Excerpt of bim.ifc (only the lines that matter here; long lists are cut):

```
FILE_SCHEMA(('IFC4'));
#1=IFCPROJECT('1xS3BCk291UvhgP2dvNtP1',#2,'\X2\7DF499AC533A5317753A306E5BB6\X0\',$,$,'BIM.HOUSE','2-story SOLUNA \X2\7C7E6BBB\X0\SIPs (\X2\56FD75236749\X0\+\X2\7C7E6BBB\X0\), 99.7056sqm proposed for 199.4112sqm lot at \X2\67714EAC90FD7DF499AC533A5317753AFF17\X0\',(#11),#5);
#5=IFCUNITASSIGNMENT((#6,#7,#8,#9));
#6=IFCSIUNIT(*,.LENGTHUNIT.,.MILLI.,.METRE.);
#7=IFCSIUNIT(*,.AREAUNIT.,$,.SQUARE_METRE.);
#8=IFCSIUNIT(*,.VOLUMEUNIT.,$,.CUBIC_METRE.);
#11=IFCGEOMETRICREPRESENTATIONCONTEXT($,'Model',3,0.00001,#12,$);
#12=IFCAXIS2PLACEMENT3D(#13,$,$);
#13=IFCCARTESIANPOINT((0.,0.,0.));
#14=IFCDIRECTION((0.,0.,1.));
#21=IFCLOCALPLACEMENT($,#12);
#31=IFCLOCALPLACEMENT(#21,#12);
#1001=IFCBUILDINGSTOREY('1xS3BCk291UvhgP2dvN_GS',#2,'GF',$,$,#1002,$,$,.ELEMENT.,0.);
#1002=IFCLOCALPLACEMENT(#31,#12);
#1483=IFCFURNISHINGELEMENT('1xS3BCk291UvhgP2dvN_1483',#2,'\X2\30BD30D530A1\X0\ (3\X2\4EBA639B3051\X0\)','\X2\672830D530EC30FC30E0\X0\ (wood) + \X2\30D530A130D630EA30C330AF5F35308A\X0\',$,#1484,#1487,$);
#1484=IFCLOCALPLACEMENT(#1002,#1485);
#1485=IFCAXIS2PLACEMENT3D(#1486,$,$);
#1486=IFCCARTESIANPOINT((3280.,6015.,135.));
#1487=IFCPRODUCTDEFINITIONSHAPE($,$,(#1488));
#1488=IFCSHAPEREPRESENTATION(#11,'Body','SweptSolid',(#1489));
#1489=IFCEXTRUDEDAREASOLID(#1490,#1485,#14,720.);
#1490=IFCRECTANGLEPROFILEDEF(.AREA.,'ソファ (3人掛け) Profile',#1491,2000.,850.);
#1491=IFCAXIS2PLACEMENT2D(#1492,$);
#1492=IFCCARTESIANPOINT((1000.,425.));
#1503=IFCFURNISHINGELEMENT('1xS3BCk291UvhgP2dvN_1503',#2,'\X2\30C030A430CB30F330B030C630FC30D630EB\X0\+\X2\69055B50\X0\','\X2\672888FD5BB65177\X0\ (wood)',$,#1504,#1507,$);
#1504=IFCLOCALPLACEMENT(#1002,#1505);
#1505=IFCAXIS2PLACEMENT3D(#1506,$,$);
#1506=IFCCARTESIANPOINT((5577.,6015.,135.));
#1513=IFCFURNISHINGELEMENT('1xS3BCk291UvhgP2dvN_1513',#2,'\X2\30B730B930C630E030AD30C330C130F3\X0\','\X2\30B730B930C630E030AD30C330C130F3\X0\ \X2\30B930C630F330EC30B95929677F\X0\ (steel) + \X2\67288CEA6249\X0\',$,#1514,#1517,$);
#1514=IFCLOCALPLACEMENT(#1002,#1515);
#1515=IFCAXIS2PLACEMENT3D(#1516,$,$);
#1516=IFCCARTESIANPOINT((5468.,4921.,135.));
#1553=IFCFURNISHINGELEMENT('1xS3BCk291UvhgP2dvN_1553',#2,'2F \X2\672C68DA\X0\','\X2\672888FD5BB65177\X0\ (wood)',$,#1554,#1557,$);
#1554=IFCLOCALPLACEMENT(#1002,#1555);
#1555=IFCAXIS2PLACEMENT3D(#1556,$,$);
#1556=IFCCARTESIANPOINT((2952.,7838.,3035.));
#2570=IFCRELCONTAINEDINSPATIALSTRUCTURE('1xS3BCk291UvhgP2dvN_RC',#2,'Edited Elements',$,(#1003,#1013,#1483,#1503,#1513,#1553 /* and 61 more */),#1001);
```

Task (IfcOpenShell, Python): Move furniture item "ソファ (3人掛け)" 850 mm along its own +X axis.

```python
import ifcopenshell
import ifcopenshell.api.geometry
import ifcopenshell.util.placement
import ifcopenshell.util.unit

model = ifcopenshell.open("bim.ifc")
unit_scale = ifcopenshell.util.unit.calculate_unit_scale(model)

item = model.by_guid("1xS3BCk291UvhgP2dvN_1483")
matrix = ifcopenshell.util.placement.get_local_placement(item.ObjectPlacement)
matrix[:3, 3] += matrix[:3, 0] * 0.85 / unit_scale
ifcopenshell.api.geometry.edit_object_placement(model, product=item, matrix=matrix, is_si=False)

print(ifcopenshell.util.placement.get_local_placement(item.ObjectPlacement).round(3) + 0.0)

model.write("bim_updated.ifc")
```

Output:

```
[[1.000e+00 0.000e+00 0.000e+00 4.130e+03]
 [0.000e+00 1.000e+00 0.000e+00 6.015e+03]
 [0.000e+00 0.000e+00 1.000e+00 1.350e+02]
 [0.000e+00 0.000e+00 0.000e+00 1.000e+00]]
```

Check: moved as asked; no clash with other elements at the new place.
